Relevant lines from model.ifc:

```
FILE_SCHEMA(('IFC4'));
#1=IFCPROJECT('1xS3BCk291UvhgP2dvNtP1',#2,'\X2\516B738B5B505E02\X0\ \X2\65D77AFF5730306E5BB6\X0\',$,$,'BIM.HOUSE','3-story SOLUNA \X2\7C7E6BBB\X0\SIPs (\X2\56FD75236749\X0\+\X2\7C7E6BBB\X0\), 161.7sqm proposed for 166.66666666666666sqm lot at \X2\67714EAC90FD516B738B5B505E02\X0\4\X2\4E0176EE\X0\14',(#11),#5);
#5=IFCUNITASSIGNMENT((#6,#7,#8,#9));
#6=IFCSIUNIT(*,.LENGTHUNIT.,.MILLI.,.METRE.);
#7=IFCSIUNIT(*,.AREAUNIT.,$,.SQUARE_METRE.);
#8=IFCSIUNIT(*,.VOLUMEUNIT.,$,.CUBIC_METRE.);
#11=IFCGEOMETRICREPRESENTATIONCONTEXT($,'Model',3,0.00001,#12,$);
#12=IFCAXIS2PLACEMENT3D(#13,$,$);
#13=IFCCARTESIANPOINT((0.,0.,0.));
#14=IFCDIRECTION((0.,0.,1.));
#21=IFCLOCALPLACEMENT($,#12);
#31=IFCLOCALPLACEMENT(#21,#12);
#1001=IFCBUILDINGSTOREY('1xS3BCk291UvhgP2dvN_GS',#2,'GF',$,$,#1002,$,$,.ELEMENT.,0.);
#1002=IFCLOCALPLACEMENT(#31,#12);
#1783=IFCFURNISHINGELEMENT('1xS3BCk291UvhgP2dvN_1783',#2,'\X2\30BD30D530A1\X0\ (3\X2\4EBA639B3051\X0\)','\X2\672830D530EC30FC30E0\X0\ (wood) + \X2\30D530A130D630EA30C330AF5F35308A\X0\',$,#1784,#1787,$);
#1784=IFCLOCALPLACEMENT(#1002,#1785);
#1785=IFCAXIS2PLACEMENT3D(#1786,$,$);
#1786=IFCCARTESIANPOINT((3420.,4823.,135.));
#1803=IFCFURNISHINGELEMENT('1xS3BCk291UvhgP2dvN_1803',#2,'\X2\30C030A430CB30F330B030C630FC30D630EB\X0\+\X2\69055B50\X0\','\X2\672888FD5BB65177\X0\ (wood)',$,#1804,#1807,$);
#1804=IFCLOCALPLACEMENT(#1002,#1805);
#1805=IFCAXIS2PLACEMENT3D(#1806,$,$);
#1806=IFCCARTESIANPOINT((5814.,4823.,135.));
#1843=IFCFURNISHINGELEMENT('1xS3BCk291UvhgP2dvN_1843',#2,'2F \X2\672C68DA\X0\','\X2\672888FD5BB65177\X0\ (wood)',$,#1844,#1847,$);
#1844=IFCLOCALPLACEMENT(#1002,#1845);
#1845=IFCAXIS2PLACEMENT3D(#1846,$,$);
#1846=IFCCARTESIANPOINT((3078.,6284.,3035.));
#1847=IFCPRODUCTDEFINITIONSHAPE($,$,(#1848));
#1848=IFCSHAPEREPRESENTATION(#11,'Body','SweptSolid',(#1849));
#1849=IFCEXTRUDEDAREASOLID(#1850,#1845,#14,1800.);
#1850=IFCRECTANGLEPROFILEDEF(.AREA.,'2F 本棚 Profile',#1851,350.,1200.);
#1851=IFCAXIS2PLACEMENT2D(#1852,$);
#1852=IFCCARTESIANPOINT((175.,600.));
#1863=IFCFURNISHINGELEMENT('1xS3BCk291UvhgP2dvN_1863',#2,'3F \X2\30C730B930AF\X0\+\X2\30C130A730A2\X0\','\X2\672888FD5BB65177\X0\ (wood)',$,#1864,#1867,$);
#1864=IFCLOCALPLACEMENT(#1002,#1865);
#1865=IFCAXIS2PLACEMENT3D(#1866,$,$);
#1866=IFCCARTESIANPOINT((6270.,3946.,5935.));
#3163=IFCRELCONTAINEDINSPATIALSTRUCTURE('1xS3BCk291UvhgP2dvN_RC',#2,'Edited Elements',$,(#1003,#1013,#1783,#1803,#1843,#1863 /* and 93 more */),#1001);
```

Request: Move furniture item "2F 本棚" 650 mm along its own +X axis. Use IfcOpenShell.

```python
import ifcopenshell
import ifcopenshell.api.geometry
import ifcopenshell.util.placement
import ifcopenshell.util.unit

model = ifcopenshell.open("model.ifc")
unit_scale = ifcopenshell.util.unit.calculate_unit_scale(model)

item = model.by_id(1843)
matrix = ifcopenshell.util.placement.get_local_placement(item.ObjectPlacement)
matrix[:3, 3] += matrix[:3, 0] * 0.65 / unit_scale
ifcopenshell.api.geometry.edit_object_placement(model, product=item, matrix=matrix, is_si=False)

print(ifcopenshell.util.placement.get_local_placement(item.ObjectPlacement).round(3) + 0.0)

model.write("model-out.ifc")
```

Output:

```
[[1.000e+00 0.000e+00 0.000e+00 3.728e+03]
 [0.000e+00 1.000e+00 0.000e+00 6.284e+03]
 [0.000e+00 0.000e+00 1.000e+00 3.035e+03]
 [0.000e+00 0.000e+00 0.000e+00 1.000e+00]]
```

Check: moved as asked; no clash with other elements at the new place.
